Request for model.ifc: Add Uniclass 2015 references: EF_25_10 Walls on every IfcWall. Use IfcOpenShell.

First a look at what the model holds.

```python
import ifcopenshell

model = ifcopenshell.open("model.ifc")
print(model.schema)
print("classifications:", [c.Name for c in model.by_type("IfcClassification")])
for ifc_class in ("IfcDoor", "IfcRoof", "IfcStair", "IfcWall", "IfcWindow"):
    print(ifc_class, len(model.by_type(ifc_class)))
```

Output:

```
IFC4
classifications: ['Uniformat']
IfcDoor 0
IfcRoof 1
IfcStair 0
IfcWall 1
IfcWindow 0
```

```python
import ifcopenshell
import ifcopenshell.api.classification

model = ifcopenshell.open("model.ifc")

system = ifcopenshell.api.classification.add_classification(model, classification="Uniclass 2015")

codes = {
    "IfcWall": ("EF_25_10", "Walls"),
}
for ifc_class, (code, name) in codes.items():
    products = model.by_type(ifc_class)
    ifcopenshell.api.classification.add_reference(
        model, products=products, classification=system, identification=code, name=name
    )
    print(code, len(products))

model.write("model_updated.ifc")
```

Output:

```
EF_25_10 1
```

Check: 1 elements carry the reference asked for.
